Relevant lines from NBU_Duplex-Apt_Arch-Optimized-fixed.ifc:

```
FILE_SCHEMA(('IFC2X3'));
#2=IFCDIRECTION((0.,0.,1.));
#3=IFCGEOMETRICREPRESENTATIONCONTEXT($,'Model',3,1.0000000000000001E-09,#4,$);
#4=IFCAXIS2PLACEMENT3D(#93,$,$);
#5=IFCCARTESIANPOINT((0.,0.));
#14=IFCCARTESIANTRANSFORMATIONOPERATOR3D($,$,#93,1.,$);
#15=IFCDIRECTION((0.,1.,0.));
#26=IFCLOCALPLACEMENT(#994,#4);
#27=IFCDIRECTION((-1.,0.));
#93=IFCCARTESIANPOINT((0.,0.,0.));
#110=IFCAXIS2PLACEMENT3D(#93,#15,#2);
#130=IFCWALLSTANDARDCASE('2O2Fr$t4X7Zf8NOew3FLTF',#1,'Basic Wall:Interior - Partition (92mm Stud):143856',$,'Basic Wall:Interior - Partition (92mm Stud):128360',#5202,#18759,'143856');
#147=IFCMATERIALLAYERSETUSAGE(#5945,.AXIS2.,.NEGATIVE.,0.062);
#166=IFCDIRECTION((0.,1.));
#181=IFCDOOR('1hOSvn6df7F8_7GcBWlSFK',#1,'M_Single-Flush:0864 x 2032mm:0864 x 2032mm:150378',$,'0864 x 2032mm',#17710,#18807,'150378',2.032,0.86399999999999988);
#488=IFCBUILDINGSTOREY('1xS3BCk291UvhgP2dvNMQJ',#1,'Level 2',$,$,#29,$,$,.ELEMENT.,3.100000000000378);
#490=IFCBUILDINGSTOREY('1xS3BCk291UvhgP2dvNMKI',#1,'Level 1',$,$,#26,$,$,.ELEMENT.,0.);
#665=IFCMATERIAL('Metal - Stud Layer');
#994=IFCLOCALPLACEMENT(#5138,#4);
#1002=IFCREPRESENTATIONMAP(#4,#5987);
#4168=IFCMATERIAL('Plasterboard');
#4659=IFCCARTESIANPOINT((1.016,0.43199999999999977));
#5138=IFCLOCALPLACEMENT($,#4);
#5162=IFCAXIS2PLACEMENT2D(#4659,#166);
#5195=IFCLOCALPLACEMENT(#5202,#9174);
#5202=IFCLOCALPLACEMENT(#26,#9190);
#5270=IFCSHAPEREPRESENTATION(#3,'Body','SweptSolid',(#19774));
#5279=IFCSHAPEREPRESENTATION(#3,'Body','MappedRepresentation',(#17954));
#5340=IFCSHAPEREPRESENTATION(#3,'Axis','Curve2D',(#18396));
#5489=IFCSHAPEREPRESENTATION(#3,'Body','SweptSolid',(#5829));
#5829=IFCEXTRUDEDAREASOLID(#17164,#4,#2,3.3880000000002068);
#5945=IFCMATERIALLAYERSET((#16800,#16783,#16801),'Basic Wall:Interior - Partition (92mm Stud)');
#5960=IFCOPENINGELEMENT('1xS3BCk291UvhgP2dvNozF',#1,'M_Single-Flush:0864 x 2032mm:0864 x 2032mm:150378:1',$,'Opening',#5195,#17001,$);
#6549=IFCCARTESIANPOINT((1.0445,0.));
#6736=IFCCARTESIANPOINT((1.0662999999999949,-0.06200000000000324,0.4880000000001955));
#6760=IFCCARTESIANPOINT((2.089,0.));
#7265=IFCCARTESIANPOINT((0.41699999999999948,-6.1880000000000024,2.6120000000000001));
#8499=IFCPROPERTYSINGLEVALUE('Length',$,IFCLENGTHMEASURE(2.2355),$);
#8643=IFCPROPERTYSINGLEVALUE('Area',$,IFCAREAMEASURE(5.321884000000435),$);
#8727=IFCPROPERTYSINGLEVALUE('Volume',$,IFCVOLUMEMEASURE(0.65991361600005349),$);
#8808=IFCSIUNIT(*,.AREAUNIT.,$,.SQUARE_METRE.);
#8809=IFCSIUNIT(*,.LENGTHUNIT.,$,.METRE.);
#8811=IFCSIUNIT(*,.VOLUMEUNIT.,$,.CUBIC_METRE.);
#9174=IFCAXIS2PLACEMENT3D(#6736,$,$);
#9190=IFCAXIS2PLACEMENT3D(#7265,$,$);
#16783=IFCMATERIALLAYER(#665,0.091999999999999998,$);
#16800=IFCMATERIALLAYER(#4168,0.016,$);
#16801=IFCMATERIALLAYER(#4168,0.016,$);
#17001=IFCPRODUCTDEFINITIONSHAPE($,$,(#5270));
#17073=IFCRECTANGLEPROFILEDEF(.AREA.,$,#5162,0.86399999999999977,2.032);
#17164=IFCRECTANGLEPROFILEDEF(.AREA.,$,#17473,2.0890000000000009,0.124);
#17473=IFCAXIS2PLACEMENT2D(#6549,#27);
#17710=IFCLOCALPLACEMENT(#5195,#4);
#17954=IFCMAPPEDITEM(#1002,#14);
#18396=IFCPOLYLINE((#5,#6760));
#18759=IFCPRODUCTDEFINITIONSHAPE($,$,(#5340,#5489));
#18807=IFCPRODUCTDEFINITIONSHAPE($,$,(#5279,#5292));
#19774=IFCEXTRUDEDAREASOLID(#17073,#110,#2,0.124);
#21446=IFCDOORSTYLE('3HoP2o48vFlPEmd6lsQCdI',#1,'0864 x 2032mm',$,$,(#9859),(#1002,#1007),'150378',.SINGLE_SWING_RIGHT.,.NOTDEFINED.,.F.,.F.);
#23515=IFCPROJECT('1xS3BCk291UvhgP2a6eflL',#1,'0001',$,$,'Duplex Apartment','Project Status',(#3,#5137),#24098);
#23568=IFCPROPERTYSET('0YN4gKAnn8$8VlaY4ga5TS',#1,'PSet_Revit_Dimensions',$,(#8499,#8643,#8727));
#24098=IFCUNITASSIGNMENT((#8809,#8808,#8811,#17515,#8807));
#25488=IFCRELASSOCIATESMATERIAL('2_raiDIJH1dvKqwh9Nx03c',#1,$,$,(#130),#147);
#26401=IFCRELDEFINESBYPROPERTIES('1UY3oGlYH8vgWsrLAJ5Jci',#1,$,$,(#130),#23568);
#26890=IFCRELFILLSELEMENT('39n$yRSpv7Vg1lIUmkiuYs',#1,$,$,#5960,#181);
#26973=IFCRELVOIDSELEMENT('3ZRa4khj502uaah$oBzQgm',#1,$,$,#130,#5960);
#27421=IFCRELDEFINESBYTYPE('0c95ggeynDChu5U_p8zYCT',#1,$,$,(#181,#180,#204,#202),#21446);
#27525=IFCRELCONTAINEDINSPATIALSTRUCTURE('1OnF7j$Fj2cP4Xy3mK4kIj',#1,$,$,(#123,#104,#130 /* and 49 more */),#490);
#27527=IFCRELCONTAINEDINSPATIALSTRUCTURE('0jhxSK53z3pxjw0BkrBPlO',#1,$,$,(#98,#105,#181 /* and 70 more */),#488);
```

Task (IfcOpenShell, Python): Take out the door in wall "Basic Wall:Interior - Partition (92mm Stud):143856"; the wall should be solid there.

```python
import ifcopenshell
import ifcopenshell.api.feature
import ifcopenshell.api.pset
import ifcopenshell.api.root
import ifcopenshell.geom
import ifcopenshell.util.element
import ifcopenshell.util.shape
import ifcopenshell.util.unit

model = ifcopenshell.open("NBU_Duplex-Apt_Arch-Optimized-fixed.ifc")
area_scale = ifcopenshell.util.unit.calculate_unit_scale(model, "AREAUNIT")
volume_scale = ifcopenshell.util.unit.calculate_unit_scale(model, "VOLUMEUNIT")
settings = ifcopenshell.geom.settings()


def volume(element):
    """Net volume in cubic metres, openings subtracted."""
    shape = ifcopenshell.geom.create_shape(settings, element)
    return ifcopenshell.util.shape.get_volume(shape.geometry)


door = model.by_guid("1hOSvn6df7F8_7GcBWlSFK")
opening = door.FillsVoids[0].RelatingOpeningElement
wall = opening.VoidsElements[0].RelatingBuildingElement
before = volume(wall)

ifcopenshell.api.root.remove_product(model, product=door)
ifcopenshell.api.feature.remove_feature(model, feature=opening)

after = volume(wall)
thickness = 0.124  # wall thickness in metres

# Update the wall's stored quantities.
pset = model.by_id(ifcopenshell.util.element.get_pset(wall, "PSet_Revit_Dimensions", should_inherit=False)["id"])
ifcopenshell.api.pset.edit_pset(model, pset=pset, properties={
    "Area": model.create_entity("IfcAreaMeasure", after / thickness / area_scale),
    "Volume": model.create_entity("IfcVolumeMeasure", after / volume_scale),
})

print(f"wall volume {before:.3f} -> {after:.3f} m3")

model.write("NBU_Duplex-Apt_Arch-Optimized-fixed-out.ifc")
```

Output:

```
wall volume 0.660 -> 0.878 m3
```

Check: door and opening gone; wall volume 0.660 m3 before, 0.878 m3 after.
